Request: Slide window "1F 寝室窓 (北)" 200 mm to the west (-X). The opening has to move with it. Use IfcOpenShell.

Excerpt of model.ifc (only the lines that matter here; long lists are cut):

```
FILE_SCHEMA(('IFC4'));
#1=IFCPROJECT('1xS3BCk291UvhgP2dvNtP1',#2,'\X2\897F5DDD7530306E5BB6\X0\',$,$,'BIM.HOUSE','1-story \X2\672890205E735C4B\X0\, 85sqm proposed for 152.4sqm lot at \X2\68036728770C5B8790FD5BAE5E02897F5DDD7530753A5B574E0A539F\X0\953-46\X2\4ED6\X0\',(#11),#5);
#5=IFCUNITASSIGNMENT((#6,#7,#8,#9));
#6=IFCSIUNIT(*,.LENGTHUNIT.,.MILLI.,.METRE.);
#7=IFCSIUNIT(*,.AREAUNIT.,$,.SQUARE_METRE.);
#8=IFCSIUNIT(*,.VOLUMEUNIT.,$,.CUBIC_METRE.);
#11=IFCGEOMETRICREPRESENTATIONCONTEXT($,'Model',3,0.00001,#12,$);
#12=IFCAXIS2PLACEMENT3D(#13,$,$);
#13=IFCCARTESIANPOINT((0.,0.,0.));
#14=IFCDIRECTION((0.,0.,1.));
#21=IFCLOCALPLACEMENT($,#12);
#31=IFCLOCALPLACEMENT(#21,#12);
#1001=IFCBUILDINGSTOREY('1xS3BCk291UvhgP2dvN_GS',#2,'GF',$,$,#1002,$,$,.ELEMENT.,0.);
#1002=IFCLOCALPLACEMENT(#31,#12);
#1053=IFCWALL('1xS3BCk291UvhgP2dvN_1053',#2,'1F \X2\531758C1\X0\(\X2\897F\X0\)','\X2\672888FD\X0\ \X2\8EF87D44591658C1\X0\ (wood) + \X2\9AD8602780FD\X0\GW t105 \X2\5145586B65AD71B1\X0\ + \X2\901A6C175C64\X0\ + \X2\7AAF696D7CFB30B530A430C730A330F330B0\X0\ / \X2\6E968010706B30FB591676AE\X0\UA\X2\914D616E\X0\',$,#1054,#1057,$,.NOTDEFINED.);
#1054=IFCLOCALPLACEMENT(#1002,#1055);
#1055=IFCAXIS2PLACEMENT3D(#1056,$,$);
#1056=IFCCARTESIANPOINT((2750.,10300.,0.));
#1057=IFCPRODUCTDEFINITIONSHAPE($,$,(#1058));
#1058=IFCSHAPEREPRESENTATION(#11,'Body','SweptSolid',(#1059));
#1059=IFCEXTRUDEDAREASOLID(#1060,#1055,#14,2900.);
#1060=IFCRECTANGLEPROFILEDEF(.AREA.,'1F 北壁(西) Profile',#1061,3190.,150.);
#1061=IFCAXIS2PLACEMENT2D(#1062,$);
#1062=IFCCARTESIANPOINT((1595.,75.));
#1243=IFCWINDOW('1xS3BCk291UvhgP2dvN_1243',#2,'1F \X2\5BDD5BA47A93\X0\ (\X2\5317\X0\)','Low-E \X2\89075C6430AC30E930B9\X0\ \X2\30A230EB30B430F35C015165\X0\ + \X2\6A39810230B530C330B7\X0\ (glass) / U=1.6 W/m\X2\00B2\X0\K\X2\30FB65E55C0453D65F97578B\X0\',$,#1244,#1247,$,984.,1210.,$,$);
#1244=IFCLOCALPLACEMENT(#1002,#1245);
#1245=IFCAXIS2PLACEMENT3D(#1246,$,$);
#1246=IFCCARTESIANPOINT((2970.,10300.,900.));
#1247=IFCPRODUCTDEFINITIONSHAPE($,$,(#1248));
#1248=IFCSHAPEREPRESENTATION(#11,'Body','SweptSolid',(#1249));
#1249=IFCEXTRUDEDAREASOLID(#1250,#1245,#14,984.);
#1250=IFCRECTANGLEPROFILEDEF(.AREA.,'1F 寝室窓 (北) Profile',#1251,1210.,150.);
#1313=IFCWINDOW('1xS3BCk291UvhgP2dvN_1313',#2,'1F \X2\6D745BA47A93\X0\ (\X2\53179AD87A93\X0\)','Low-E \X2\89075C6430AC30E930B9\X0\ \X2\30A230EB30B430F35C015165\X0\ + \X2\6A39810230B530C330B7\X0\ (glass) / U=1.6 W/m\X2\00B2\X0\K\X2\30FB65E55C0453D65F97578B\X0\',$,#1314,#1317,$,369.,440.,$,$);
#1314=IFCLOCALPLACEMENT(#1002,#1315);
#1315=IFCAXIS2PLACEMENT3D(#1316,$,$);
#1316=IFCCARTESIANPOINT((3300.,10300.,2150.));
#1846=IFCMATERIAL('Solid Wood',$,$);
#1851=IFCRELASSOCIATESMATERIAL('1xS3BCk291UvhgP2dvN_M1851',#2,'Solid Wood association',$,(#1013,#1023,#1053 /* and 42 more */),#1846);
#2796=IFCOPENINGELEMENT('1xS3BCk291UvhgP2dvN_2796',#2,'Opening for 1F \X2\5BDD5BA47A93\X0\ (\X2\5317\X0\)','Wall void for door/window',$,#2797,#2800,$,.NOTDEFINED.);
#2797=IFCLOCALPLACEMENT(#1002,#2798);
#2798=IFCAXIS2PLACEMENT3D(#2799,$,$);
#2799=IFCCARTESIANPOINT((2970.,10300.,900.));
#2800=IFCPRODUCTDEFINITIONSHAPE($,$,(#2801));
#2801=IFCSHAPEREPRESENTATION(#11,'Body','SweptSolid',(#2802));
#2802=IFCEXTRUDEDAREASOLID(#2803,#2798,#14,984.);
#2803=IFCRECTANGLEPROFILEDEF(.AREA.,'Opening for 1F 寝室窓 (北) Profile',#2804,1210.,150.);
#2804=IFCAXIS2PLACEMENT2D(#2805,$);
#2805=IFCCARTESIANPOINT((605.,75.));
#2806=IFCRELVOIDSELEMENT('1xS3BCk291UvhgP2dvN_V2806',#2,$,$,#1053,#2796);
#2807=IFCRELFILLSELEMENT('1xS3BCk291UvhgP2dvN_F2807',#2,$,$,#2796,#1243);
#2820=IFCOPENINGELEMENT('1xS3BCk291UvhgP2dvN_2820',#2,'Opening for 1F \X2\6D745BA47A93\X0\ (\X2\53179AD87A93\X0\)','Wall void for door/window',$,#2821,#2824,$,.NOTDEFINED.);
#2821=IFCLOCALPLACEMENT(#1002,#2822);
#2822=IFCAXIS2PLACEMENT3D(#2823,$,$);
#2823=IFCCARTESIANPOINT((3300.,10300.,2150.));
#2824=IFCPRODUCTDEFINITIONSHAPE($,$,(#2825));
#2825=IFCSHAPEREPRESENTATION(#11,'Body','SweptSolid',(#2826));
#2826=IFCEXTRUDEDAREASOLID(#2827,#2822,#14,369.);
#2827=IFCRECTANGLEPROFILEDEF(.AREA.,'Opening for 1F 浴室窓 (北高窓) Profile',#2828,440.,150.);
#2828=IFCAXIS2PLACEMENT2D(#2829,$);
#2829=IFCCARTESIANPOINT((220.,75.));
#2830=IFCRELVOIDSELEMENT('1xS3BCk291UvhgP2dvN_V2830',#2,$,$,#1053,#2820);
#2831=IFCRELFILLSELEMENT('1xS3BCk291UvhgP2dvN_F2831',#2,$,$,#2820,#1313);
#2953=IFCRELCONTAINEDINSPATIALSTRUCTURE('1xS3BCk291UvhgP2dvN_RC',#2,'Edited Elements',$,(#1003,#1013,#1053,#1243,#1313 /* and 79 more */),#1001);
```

```python
import ifcopenshell
import ifcopenshell.api.geometry
import ifcopenshell.util.placement

model = ifcopenshell.open("model.ifc")

window = model.by_id(1243)
opening = window.FillsVoids[0].RelatingOpeningElement
wall = opening.VoidsElements[0].RelatingBuildingElement

wall_matrix = ifcopenshell.util.placement.get_local_placement(wall.ObjectPlacement)
shift = wall_matrix[:3, 0] * -200.0
before = ifcopenshell.util.placement.get_local_placement(window.ObjectPlacement)[:3, 3].copy()

# The window is not placed relative to its opening, so move both.
for product in (opening, window):
    matrix = ifcopenshell.util.placement.get_local_placement(product.ObjectPlacement)
    matrix[:3, 3] += shift
    ifcopenshell.api.geometry.edit_object_placement(model, product=product, matrix=matrix, is_si=False)

after = ifcopenshell.util.placement.get_local_placement(window.ObjectPlacement)[:3, 3]
print("window moved by", (after - before).round(3) + 0.0)

model.write("model_v2.ifc")
```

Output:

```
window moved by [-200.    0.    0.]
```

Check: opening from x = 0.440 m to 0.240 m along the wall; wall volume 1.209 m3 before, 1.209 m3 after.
